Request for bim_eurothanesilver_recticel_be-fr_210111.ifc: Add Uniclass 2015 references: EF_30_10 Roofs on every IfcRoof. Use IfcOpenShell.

First a look at what the model holds.

```python
import ifcopenshell

model = ifcopenshell.open("bim_eurothanesilver_recticel_be-fr_210111.ifc")
print(model.schema)
print("classifications:", [c.Name for c in model.by_type("IfcClassification")])
for ifc_class in ("IfcDoor", "IfcRoof", "IfcStair", "IfcWall", "IfcWindow"):
    print(ifc_class, len(model.by_type(ifc_class)))
```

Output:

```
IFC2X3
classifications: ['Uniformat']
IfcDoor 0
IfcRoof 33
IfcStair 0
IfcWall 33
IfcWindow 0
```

```python
import ifcopenshell
import ifcopenshell.api.classification

model = ifcopenshell.open("bim_eurothanesilver_recticel_be-fr_210111.ifc")

# IFC2X3 requires Source and Edition and has no link from the project to the system.
system = model.create_entity("IfcClassification", Source="NBS", Edition="2015", Name="Uniclass 2015")

codes = {
    "IfcRoof": ("EF_30_10", "Roofs"),
}
for ifc_class, (code, name) in codes.items():
    products = model.by_type(ifc_class)
    ifcopenshell.api.classification.add_reference(
        model, products=products, classification=system, identification=code, name=name
    )
    print(code, len(products))

model.write("bim_eurothanesilver_recticel_be-fr_210111_v2.ifc")
```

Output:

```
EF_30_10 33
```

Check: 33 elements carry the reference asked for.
